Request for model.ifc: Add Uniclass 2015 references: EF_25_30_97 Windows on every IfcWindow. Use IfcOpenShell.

First a look at what the model holds.

```python
import ifcopenshell

model = ifcopenshell.open("model.ifc")
print(model.schema)
print("classifications:", [c.Name for c in model.by_type("IfcClassification")])
for ifc_class in ("IfcDoor", "IfcRoof", "IfcStair", "IfcWall", "IfcWindow"):
    print(ifc_class, len(model.by_type(ifc_class)))
```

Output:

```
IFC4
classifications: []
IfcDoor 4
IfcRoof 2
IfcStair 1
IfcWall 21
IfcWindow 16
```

```python
import ifcopenshell
import ifcopenshell.api.classification

model = ifcopenshell.open("model.ifc")

system = ifcopenshell.api.classification.add_classification(model, classification="Uniclass 2015")

codes = {
    "IfcWindow": ("EF_25_30_97", "Windows"),
}
for ifc_class, (code, name) in codes.items():
    products = model.by_type(ifc_class)
    ifcopenshell.api.classification.add_reference(
        model, products=products, classification=system, identification=code, name=name
    )
    print(code, len(products))

model.write("model_edited.ifc")
```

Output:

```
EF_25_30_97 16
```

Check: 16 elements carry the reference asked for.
